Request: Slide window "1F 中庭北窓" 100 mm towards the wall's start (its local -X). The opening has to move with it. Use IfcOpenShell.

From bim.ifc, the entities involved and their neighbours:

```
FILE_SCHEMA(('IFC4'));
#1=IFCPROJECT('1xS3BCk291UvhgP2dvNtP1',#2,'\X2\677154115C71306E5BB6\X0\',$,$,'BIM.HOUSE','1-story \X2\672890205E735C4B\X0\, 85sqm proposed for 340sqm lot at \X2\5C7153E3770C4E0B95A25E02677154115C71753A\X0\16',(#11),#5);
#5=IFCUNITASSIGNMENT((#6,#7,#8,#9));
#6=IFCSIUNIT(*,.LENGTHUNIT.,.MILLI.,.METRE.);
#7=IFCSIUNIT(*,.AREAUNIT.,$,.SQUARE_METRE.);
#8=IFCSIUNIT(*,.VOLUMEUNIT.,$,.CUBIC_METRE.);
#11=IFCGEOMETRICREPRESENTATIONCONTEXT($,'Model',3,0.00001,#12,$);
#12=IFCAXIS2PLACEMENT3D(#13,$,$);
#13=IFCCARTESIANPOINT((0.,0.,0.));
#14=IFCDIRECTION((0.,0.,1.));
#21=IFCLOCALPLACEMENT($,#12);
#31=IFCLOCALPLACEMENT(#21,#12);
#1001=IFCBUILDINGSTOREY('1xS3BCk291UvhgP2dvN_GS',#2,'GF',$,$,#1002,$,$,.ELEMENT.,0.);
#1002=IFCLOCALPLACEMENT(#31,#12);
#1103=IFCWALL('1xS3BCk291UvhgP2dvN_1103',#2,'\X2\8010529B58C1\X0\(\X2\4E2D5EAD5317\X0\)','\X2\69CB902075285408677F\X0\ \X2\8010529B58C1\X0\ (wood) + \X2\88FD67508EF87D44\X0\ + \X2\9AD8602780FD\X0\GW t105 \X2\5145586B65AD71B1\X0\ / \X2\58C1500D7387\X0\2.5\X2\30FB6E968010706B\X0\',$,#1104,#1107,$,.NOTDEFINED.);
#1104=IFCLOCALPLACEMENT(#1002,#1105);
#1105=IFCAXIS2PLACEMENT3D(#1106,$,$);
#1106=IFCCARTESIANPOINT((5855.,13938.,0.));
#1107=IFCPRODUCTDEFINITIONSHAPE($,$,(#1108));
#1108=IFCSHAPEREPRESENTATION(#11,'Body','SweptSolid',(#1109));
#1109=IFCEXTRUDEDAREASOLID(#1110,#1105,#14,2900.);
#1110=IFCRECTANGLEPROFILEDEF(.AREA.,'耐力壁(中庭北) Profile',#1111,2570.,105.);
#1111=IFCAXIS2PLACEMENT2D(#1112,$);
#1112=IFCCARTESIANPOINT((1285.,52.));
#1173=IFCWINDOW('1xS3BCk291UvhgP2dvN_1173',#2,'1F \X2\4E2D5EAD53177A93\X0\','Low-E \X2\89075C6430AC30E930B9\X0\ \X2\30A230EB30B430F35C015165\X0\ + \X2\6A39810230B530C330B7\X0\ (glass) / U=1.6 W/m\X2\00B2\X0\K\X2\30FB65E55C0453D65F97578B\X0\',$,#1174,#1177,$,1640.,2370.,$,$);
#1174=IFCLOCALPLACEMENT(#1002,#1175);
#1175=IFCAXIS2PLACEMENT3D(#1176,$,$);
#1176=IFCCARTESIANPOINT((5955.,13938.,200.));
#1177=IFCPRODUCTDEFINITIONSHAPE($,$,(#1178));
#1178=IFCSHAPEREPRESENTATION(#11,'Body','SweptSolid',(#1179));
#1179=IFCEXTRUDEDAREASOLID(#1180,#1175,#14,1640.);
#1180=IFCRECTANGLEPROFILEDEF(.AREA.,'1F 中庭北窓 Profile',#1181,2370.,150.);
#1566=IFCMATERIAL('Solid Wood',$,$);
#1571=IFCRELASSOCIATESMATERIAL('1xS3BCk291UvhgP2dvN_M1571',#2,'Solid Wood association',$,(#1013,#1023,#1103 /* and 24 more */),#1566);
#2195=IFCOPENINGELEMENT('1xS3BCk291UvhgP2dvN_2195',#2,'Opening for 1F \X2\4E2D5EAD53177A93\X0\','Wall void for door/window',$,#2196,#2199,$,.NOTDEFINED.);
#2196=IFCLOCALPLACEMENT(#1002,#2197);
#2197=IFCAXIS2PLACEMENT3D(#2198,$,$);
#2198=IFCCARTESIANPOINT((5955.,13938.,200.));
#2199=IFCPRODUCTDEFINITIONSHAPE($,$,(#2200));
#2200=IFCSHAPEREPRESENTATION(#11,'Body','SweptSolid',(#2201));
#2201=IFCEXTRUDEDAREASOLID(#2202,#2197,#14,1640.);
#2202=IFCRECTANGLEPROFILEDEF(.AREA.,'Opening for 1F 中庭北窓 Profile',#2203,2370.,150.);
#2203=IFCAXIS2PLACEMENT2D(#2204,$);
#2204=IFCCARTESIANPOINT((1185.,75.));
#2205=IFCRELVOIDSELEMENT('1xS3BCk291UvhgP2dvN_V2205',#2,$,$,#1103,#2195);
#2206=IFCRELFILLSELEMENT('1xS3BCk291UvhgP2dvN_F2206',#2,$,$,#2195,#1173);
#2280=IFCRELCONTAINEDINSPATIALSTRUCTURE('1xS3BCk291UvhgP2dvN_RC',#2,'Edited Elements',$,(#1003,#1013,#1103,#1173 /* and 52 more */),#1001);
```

```python
import ifcopenshell
import ifcopenshell.api.geometry
import ifcopenshell.util.placement
import ifcopenshell.util.unit

model = ifcopenshell.open("bim.ifc")
unit_scale = ifcopenshell.util.unit.calculate_unit_scale(model)

window = model.by_guid("1xS3BCk291UvhgP2dvN_1173")
opening = window.FillsVoids[0].RelatingOpeningElement
wall = opening.VoidsElements[0].RelatingBuildingElement

wall_matrix = ifcopenshell.util.placement.get_local_placement(wall.ObjectPlacement)
shift = wall_matrix[:3, 0] * -0.1 / unit_scale
before = ifcopenshell.util.placement.get_local_placement(window.ObjectPlacement)[:3, 3].copy()

# The window is not placed relative to its opening, so move both.
for product in (opening, window):
    matrix = ifcopenshell.util.placement.get_local_placement(product.ObjectPlacement)
    matrix[:3, 3] += shift
    ifcopenshell.api.geometry.edit_object_placement(model, product=product, matrix=matrix, is_si=False)

after = ifcopenshell.util.placement.get_local_placement(window.ObjectPlacement)[:3, 3]
print("window moved by", (after - before).round(3) + 0.0)

model.write("bim_updated.ifc")
```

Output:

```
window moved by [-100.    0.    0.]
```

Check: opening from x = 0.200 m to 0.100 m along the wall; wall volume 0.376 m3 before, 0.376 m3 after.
